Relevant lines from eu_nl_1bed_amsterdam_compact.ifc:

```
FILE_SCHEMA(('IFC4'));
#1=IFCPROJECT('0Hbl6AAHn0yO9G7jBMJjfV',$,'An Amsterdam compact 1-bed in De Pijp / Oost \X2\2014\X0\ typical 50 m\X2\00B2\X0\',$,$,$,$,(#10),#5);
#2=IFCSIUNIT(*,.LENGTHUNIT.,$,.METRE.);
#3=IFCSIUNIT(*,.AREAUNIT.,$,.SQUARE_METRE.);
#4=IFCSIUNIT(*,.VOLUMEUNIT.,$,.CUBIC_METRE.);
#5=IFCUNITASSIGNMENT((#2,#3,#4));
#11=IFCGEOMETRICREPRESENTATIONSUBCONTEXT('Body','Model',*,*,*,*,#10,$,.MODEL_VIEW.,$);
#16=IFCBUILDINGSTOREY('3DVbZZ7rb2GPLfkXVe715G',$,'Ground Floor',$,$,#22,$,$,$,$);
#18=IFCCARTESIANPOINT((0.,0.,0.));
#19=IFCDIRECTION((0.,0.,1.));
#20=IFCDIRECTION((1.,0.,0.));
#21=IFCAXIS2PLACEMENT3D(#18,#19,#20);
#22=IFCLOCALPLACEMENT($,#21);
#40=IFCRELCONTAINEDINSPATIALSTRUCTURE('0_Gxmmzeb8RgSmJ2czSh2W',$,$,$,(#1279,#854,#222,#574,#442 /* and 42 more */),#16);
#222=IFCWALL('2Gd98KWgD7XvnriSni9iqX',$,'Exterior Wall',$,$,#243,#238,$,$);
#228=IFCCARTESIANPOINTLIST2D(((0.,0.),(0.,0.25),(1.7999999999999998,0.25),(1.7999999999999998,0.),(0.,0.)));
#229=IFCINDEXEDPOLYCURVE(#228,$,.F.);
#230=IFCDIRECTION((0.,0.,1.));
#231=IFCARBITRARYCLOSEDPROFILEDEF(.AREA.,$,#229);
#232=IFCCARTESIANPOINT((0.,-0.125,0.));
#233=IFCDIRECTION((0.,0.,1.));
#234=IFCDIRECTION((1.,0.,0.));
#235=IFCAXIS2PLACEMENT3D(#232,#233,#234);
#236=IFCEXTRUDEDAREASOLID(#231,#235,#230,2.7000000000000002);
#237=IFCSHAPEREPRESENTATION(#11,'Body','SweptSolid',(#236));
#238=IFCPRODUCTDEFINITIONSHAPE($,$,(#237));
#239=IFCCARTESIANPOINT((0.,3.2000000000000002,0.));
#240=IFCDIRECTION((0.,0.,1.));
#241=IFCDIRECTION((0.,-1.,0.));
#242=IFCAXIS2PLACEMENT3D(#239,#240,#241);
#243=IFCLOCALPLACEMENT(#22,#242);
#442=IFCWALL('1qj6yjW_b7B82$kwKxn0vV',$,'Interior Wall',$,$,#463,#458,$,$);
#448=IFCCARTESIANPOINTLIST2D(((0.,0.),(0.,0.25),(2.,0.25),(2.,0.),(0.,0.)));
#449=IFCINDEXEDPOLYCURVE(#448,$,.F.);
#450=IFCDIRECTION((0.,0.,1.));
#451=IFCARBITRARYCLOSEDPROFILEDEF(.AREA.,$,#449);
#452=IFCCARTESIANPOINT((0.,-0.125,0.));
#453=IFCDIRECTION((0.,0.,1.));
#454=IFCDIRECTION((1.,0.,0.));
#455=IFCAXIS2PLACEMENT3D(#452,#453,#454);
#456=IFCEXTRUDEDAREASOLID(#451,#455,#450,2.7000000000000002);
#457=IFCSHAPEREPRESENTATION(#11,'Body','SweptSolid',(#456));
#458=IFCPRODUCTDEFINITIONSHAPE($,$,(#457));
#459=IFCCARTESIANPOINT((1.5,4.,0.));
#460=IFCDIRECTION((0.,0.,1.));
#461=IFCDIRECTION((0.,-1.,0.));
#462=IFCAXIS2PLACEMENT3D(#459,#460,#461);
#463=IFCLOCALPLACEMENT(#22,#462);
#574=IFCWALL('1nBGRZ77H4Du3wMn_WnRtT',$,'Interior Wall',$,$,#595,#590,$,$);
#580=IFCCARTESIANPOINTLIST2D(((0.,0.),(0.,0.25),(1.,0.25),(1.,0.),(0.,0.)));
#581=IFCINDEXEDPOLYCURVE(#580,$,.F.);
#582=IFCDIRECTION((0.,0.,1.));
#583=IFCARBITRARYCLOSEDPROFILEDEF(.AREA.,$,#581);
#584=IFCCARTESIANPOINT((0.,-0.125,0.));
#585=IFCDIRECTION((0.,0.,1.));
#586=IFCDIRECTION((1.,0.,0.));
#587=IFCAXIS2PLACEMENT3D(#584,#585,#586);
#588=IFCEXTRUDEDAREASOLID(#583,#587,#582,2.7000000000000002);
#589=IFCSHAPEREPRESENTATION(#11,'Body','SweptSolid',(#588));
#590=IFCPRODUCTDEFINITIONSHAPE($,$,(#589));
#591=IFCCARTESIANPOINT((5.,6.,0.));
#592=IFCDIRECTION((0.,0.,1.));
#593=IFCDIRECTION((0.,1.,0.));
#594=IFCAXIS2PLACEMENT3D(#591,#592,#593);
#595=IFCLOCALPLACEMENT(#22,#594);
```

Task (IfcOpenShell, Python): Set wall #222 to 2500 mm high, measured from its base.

```python
import ifcopenshell
import ifcopenshell.geom
import ifcopenshell.util.representation
import ifcopenshell.util.shape

model = ifcopenshell.open("eu_nl_1bed_amsterdam_compact.ifc")
settings = ifcopenshell.geom.settings()


def volume(element):
    """Net volume in cubic metres, openings subtracted."""
    shape = ifcopenshell.geom.create_shape(settings, element)
    return ifcopenshell.util.shape.get_volume(shape.geometry)


wall = model.by_guid("2Gd98KWgD7XvnriSni9iqX")
before = volume(wall)

body = ifcopenshell.util.representation.get_representation(wall, "Model", "Body")
solid = body.Items[0]
old_height = solid.Depth
solid.Depth = 2.5
after = volume(wall)

print(f"height {old_height:g} -> {solid.Depth:g}, volume {before:.3f} -> {after:.3f} m3")

model.write("eu_nl_1bed_amsterdam_compact_updated.ifc")
```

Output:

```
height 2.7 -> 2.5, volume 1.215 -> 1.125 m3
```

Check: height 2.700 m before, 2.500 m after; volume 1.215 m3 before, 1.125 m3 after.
